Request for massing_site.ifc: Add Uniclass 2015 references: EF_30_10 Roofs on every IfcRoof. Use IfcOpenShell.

First a look at what the model holds.

```python
import ifcopenshell

model = ifcopenshell.open("massing_site.ifc")
print(model.schema)
print("classifications:", [c.Name for c in model.by_type("IfcClassification")])
for ifc_class in ("IfcDoor", "IfcRoof", "IfcStair", "IfcWall", "IfcWindow"):
    print(ifc_class, len(model.by_type(ifc_class)))
```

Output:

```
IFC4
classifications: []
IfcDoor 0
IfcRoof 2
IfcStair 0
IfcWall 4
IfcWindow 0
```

```python
import ifcopenshell
import ifcopenshell.api.classification

model = ifcopenshell.open("massing_site.ifc")

system = ifcopenshell.api.classification.add_classification(model, classification="Uniclass 2015")

codes = {
    "IfcRoof": ("EF_30_10", "Roofs"),
}
for ifc_class, (code, name) in codes.items():
    products = model.by_type(ifc_class)
    ifcopenshell.api.classification.add_reference(
        model, products=products, classification=system, identification=code, name=name
    )
    print(code, len(products))

model.write("massing_site_v2.ifc")
```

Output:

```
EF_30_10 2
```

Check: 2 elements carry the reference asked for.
